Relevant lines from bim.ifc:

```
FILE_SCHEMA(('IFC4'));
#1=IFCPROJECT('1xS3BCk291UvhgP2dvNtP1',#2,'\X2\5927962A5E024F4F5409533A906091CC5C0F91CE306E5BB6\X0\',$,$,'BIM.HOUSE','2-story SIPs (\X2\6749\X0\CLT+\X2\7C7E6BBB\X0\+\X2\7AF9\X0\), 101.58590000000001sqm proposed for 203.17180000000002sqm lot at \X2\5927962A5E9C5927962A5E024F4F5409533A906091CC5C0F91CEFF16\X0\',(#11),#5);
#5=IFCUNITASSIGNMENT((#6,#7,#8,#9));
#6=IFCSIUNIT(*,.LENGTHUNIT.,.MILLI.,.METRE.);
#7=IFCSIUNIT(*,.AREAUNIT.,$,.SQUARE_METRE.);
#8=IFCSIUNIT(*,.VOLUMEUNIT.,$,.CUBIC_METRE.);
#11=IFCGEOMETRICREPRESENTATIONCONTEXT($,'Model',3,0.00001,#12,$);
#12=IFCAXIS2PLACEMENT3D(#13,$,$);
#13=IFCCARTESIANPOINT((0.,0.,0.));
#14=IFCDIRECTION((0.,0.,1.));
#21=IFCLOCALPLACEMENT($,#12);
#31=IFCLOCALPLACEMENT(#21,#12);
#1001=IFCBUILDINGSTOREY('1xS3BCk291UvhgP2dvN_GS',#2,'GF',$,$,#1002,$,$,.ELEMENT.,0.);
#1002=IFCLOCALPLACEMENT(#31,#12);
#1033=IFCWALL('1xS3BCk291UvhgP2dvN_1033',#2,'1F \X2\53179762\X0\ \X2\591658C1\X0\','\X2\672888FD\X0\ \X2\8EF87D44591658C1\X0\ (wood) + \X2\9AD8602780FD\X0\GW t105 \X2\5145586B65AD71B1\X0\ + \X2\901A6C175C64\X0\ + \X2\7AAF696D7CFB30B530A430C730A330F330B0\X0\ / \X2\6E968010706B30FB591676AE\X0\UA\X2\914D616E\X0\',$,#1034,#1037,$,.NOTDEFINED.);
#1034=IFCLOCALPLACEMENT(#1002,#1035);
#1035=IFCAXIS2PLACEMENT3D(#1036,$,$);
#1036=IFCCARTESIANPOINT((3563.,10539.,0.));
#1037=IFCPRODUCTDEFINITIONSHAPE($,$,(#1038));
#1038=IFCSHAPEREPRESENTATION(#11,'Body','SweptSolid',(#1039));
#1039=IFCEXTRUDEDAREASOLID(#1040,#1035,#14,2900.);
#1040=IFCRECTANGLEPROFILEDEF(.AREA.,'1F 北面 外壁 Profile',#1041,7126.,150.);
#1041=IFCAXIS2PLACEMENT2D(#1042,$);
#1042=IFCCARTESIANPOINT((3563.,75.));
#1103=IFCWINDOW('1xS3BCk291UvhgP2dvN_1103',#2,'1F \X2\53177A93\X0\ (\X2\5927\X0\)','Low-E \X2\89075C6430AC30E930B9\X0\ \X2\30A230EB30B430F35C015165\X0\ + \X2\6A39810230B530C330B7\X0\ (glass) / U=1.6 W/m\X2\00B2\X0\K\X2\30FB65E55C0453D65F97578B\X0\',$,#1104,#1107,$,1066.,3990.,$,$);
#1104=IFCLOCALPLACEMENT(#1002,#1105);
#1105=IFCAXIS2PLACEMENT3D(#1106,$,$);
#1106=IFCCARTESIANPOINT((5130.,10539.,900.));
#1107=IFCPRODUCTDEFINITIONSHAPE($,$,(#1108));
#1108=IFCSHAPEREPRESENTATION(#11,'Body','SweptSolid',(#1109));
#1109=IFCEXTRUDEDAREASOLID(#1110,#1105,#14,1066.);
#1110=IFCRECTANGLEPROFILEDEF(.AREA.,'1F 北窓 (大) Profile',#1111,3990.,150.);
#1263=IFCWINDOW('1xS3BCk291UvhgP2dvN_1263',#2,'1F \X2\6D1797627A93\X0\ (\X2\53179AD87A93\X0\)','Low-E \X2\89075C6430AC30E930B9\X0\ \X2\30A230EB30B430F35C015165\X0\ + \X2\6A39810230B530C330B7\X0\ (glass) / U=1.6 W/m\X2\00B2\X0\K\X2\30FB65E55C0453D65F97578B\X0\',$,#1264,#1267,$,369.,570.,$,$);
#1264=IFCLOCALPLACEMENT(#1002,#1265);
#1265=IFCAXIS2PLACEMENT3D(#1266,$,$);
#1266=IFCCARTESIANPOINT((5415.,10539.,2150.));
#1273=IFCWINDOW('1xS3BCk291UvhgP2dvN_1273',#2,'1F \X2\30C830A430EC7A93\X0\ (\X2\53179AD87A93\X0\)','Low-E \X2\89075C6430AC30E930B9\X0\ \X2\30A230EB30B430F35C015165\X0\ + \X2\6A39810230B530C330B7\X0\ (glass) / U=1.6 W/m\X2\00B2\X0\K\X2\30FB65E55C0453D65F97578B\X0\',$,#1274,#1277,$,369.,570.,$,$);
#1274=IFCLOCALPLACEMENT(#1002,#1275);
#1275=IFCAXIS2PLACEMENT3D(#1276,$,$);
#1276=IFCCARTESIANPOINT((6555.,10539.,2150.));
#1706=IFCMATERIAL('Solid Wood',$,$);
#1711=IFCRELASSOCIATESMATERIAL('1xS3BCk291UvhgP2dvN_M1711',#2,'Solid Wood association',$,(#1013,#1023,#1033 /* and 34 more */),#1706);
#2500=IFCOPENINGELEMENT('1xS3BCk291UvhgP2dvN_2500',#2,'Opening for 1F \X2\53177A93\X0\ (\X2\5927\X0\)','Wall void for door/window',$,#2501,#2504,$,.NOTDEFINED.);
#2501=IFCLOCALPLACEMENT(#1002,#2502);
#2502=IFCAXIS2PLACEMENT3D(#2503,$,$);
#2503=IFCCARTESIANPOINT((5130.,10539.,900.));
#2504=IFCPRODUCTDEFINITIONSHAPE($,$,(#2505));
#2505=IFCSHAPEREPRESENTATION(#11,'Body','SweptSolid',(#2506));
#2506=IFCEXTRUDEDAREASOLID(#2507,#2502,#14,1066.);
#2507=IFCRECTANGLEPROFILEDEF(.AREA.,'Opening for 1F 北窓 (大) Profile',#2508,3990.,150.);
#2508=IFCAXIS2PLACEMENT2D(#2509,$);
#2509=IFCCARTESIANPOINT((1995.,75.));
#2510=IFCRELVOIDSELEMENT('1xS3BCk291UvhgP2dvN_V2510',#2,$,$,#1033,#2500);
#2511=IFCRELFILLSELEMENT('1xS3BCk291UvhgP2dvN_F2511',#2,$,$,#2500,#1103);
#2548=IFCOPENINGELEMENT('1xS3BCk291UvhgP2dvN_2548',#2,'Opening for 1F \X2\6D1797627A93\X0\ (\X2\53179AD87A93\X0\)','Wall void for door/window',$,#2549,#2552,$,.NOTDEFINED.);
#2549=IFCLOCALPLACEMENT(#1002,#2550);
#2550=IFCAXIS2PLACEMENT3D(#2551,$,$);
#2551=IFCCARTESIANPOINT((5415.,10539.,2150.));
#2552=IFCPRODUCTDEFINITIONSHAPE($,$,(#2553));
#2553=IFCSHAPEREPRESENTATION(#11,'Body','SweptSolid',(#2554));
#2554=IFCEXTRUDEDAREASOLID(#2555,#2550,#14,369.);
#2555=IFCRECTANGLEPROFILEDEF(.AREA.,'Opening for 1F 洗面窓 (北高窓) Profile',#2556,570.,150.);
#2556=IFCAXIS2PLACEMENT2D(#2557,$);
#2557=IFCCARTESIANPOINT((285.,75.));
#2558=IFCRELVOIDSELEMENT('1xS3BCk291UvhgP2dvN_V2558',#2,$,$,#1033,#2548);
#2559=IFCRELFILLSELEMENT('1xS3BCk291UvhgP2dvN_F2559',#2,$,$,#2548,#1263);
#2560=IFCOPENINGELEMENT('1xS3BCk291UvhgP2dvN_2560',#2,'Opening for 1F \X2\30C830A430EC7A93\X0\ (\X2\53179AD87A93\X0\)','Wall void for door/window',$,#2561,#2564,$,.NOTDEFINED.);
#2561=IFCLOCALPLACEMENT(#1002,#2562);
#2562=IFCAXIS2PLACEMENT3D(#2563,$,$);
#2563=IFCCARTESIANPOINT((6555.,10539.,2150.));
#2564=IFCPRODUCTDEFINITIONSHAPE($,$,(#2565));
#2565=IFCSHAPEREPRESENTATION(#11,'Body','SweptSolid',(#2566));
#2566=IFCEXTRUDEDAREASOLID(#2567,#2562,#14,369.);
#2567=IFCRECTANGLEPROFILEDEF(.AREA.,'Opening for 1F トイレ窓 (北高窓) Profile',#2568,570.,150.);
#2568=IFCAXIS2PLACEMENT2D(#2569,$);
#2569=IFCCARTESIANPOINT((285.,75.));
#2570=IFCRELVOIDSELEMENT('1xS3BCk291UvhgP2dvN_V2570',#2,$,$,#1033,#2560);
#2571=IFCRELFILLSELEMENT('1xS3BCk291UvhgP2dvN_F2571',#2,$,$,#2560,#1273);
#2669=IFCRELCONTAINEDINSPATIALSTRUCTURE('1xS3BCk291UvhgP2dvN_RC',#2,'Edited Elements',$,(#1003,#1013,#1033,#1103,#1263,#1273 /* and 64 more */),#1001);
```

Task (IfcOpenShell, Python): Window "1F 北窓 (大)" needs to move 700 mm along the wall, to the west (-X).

```python
import ifcopenshell
import ifcopenshell.api.geometry
import ifcopenshell.util.placement

model = ifcopenshell.open("bim.ifc")

window = model.by_guid("1xS3BCk291UvhgP2dvN_1103")
opening = window.FillsVoids[0].RelatingOpeningElement
wall = opening.VoidsElements[0].RelatingBuildingElement

wall_matrix = ifcopenshell.util.placement.get_local_placement(wall.ObjectPlacement)
shift = wall_matrix[:3, 0] * -700.0
before = ifcopenshell.util.placement.get_local_placement(window.ObjectPlacement)[:3, 3].copy()

# The window is not placed relative to its opening, so move both.
for product in (opening, window):
    matrix = ifcopenshell.util.placement.get_local_placement(product.ObjectPlacement)
    matrix[:3, 3] += shift
    ifcopenshell.api.geometry.edit_object_placement(model, product=product, matrix=matrix, is_si=False)

after = ifcopenshell.util.placement.get_local_placement(window.ObjectPlacement)[:3, 3]
print("window moved by", (after - before).round(3) + 0.0)

model.write("bim-out.ifc")
```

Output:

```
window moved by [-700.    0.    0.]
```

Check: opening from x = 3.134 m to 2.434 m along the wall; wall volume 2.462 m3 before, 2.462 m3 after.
